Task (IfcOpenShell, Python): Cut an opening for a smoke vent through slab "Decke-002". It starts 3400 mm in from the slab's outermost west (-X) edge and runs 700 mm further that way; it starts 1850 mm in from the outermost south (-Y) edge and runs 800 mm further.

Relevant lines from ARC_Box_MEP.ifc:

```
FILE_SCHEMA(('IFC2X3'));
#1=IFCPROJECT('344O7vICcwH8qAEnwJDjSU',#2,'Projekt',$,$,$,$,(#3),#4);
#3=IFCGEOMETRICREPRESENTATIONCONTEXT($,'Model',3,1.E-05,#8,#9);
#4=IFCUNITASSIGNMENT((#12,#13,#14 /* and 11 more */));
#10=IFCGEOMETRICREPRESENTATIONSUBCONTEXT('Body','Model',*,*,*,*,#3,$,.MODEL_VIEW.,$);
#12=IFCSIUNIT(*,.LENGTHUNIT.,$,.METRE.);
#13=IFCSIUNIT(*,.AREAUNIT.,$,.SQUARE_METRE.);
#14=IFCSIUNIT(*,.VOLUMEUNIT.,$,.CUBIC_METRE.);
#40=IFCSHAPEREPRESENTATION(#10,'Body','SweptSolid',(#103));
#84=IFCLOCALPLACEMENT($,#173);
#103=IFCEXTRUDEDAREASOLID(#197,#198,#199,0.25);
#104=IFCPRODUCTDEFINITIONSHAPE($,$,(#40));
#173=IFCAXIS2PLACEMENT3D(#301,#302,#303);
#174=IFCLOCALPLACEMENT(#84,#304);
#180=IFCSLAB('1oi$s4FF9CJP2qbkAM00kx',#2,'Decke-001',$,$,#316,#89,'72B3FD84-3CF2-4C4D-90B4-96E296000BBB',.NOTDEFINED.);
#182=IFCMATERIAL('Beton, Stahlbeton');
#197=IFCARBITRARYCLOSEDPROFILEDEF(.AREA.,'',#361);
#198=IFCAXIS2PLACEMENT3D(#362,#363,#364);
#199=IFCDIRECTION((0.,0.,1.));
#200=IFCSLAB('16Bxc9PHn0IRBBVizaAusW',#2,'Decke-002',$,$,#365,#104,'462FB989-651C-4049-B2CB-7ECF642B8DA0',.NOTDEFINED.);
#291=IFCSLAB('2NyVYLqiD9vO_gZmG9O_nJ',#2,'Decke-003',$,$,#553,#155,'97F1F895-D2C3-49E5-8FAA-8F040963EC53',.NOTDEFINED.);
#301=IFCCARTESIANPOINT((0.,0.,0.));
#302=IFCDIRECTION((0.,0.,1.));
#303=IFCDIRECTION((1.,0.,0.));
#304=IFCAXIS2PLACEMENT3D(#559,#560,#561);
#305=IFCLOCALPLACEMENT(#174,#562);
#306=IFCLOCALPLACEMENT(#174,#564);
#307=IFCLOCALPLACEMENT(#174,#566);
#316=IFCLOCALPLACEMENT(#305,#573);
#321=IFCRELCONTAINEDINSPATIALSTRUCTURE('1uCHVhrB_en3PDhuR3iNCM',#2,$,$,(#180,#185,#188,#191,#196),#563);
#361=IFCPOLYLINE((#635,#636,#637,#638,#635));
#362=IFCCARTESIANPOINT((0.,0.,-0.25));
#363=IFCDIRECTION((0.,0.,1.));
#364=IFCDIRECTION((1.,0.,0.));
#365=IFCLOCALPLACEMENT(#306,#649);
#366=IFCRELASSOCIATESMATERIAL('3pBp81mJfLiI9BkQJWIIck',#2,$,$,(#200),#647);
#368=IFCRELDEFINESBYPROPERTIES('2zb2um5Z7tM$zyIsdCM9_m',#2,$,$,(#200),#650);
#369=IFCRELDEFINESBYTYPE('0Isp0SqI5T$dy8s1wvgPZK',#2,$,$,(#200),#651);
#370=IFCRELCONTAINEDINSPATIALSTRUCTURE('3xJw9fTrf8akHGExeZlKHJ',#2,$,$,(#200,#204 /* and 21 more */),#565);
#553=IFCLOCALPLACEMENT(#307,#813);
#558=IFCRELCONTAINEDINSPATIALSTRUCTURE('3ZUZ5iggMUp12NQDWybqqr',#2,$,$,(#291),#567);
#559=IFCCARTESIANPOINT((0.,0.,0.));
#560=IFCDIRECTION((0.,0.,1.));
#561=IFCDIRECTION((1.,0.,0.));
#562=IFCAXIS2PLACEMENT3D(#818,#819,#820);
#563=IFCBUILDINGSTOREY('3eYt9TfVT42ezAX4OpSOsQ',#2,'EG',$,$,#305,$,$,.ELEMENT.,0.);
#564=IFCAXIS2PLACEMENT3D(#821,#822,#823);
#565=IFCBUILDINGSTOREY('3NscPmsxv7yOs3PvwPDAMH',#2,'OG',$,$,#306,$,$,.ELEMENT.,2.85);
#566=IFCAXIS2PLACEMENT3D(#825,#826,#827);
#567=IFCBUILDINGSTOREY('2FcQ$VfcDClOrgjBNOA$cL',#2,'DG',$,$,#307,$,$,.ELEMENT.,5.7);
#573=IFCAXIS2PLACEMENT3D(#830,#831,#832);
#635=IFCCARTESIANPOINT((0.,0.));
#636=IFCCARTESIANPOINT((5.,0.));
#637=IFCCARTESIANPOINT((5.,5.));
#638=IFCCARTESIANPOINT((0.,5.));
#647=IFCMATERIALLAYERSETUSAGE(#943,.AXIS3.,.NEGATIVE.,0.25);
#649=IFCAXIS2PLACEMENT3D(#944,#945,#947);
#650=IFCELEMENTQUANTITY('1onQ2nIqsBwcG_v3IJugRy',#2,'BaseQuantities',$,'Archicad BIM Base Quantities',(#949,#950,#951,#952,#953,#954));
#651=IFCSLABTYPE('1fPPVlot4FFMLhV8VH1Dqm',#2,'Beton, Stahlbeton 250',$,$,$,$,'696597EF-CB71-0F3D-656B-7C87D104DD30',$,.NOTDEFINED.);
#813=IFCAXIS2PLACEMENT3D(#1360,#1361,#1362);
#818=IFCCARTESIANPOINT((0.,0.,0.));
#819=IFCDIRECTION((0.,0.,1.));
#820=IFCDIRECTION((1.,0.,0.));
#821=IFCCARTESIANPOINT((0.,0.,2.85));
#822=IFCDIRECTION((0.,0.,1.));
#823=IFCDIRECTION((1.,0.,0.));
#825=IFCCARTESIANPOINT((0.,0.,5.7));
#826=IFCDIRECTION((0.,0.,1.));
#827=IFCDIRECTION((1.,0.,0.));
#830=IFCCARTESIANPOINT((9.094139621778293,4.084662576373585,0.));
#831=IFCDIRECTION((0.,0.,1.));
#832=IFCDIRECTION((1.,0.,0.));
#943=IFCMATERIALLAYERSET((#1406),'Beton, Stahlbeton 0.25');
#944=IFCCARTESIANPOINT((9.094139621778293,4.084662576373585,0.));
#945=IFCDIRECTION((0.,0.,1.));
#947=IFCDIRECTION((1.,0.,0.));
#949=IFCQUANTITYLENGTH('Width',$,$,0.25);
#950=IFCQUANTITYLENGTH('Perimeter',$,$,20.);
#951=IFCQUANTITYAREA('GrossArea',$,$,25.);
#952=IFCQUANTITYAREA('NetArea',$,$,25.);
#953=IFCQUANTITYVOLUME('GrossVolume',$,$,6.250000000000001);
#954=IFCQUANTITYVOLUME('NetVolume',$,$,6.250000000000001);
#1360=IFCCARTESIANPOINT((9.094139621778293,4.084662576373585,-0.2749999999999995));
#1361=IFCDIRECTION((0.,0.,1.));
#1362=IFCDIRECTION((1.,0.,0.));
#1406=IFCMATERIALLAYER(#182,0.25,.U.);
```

```python
import numpy as np
import ifcopenshell
import ifcopenshell.api.feature
import ifcopenshell.api.geometry
import ifcopenshell.api.pset
import ifcopenshell.api.root
import ifcopenshell.geom
import ifcopenshell.util.element
import ifcopenshell.util.placement
import ifcopenshell.util.representation
import ifcopenshell.util.shape
import ifcopenshell.util.unit

model = ifcopenshell.open("ARC_Box_MEP.ifc")
unit_scale = ifcopenshell.util.unit.calculate_unit_scale(model)
area_scale = ifcopenshell.util.unit.calculate_unit_scale(model, "AREAUNIT")
volume_scale = ifcopenshell.util.unit.calculate_unit_scale(model, "VOLUMEUNIT")
settings = ifcopenshell.geom.settings()


def volume(element):
    """Net volume in cubic metres, openings subtracted."""
    shape = ifcopenshell.geom.create_shape(settings, element)
    return ifcopenshell.util.shape.get_volume(shape.geometry)


slab = model.by_id(200)
before = volume(slab)

# Extent in the slab's own axes, in metres. The edges named are its -X and -Y sides.
slab_shape = ifcopenshell.geom.create_shape(settings, slab)
vertices = ifcopenshell.util.shape.get_vertices(slab_shape.geometry)
x_min, y_min, bottom = vertices.min(axis=0)
top = vertices[:, 2].max()

opening = ifcopenshell.api.root.create_entity(model, ifc_class="IfcOpeningElement", name="Smoke vent opening")
context = ifcopenshell.util.representation.get_context(model, "Model", "Body", "MODEL_VIEW")
width, depth = 0.7, 0.8
outline = [(0.0, 0.0), (width, 0.0), (width, depth), (0.0, depth), (0.0, 0.0)]
# Overshoot both faces by 50 mm so the cut is clean.
shape = ifcopenshell.api.geometry.add_slab_representation(
    model, context=context, depth=top - bottom + 0.1, polyline=outline
)
ifcopenshell.api.geometry.assign_representation(model, product=opening, representation=shape)

matrix = ifcopenshell.util.placement.get_local_placement(slab.ObjectPlacement)
matrix[:, 3] = matrix @ np.append(np.array([x_min + 3.4, y_min + 1.85, bottom - 0.05]) / unit_scale, 1.0)
ifcopenshell.api.geometry.edit_object_placement(model, product=opening, matrix=matrix, is_si=False)
ifcopenshell.api.feature.add_feature(model, feature=opening, element=slab)

after = volume(slab)

# Update the slab's stored quantities.
qto = model.by_id(ifcopenshell.util.element.get_pset(slab, "BaseQuantities", should_inherit=False)["id"])
ifcopenshell.api.pset.edit_qto(model, qto=qto, properties={
    "NetArea": after / (top - bottom) / area_scale,
    "NetVolume": after / volume_scale,
})

print(f"slab volume {before:.3f} -> {after:.3f} m3")

model.write("ARC_Box_MEP_updated.ifc")
```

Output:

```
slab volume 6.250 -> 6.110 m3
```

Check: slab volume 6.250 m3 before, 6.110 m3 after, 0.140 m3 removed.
